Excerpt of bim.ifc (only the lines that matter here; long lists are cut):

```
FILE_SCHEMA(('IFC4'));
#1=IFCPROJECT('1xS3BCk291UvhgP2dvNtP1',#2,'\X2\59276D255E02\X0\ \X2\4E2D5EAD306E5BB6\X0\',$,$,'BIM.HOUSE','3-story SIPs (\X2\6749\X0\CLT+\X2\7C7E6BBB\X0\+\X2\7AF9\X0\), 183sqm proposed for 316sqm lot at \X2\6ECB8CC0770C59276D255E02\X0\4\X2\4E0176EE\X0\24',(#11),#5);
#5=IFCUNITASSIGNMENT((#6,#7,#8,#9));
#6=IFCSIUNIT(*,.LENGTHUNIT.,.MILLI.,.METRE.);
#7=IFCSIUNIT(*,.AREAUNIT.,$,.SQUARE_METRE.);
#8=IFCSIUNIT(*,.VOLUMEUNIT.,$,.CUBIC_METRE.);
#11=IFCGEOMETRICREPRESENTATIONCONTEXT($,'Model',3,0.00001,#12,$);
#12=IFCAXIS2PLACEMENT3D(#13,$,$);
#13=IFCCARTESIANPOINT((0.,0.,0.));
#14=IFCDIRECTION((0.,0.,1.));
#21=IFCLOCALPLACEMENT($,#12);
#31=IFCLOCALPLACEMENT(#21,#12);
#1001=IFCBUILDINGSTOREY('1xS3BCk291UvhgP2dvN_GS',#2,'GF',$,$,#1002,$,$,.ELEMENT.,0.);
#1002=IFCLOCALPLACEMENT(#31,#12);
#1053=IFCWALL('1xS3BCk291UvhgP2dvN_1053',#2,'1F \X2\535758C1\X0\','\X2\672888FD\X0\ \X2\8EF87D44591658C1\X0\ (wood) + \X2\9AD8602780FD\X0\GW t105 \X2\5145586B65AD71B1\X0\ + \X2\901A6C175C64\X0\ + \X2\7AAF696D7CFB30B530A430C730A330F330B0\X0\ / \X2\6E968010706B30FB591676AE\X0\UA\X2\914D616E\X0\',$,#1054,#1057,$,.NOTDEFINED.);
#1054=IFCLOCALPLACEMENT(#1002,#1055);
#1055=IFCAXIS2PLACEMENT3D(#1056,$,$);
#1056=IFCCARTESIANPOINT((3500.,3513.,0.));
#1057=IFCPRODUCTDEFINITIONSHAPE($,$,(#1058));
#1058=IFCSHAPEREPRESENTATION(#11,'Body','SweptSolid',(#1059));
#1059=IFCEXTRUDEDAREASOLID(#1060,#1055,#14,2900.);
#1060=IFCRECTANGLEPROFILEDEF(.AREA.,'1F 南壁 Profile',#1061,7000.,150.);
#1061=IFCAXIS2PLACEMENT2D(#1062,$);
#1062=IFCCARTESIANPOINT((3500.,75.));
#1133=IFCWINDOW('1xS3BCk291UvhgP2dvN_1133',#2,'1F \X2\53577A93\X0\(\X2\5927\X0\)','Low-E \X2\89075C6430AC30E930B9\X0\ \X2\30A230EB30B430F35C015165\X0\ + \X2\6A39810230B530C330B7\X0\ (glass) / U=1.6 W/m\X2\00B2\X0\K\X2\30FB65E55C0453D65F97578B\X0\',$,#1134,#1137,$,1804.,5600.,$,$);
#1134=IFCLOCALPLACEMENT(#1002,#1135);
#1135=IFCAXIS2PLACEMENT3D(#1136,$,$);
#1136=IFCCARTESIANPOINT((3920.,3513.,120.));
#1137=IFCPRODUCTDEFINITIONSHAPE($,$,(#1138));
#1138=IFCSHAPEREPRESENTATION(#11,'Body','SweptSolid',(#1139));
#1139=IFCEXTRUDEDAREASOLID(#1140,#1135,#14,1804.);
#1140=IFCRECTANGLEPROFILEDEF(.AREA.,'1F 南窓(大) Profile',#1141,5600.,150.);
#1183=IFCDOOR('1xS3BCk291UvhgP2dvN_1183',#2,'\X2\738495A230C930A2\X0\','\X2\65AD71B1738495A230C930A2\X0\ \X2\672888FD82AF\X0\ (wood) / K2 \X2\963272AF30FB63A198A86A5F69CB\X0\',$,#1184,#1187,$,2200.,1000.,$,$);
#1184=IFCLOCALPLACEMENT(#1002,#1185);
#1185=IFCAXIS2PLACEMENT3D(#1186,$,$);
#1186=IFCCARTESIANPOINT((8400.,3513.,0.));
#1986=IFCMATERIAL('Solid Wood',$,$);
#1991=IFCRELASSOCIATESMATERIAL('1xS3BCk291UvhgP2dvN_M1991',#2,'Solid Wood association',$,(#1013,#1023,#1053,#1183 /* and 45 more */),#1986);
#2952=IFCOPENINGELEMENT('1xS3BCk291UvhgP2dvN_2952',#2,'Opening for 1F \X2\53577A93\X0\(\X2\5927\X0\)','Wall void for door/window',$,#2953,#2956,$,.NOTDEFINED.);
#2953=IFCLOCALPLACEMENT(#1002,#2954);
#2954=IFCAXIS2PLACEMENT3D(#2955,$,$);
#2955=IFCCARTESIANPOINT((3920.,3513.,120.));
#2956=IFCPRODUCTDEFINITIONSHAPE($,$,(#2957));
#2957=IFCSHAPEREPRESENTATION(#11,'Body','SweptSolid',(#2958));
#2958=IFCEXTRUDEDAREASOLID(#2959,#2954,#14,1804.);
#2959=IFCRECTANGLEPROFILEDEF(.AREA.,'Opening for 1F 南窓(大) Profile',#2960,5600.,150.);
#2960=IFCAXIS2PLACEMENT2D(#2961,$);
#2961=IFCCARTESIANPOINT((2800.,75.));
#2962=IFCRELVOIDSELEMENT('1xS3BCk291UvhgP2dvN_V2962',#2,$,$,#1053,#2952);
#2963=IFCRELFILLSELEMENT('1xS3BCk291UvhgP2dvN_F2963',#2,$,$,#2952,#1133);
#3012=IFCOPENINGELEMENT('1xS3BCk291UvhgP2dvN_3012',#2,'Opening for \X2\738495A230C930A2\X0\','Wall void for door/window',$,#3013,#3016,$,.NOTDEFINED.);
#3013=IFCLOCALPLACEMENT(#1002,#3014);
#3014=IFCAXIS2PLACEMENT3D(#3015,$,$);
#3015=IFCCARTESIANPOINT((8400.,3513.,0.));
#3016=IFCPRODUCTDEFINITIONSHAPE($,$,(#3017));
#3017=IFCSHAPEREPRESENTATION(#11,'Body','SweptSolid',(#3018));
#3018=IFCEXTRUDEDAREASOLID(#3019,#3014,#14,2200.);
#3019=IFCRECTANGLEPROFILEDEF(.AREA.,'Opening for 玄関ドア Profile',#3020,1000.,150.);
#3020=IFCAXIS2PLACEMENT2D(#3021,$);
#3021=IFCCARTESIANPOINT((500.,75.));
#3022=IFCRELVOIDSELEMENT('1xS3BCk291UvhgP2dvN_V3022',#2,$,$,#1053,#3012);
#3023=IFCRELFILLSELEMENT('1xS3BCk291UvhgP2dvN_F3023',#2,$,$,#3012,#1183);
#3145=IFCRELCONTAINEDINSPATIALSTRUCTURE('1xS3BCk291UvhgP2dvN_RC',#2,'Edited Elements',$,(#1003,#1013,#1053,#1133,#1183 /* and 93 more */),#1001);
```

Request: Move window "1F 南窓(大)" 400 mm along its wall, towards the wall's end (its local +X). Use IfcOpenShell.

```python
import ifcopenshell
import ifcopenshell.api.geometry
import ifcopenshell.util.placement

model = ifcopenshell.open("bim.ifc")

window = model.by_id(1133)
opening = window.FillsVoids[0].RelatingOpeningElement
wall = opening.VoidsElements[0].RelatingBuildingElement

wall_matrix = ifcopenshell.util.placement.get_local_placement(wall.ObjectPlacement)
shift = wall_matrix[:3, 0] * 400.0
before = ifcopenshell.util.placement.get_local_placement(window.ObjectPlacement)[:3, 3].copy()

# The window is not placed relative to its opening, so move both.
for product in (opening, window):
    matrix = ifcopenshell.util.placement.get_local_placement(product.ObjectPlacement)
    matrix[:3, 3] += shift
    ifcopenshell.api.geometry.edit_object_placement(model, product=product, matrix=matrix, is_si=False)

after = ifcopenshell.util.placement.get_local_placement(window.ObjectPlacement)[:3, 3]
print("window moved by", (after - before).round(3) + 0.0)

model.write("bim-out.ifc")
```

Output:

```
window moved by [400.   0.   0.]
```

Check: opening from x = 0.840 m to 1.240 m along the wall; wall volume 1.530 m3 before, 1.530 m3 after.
